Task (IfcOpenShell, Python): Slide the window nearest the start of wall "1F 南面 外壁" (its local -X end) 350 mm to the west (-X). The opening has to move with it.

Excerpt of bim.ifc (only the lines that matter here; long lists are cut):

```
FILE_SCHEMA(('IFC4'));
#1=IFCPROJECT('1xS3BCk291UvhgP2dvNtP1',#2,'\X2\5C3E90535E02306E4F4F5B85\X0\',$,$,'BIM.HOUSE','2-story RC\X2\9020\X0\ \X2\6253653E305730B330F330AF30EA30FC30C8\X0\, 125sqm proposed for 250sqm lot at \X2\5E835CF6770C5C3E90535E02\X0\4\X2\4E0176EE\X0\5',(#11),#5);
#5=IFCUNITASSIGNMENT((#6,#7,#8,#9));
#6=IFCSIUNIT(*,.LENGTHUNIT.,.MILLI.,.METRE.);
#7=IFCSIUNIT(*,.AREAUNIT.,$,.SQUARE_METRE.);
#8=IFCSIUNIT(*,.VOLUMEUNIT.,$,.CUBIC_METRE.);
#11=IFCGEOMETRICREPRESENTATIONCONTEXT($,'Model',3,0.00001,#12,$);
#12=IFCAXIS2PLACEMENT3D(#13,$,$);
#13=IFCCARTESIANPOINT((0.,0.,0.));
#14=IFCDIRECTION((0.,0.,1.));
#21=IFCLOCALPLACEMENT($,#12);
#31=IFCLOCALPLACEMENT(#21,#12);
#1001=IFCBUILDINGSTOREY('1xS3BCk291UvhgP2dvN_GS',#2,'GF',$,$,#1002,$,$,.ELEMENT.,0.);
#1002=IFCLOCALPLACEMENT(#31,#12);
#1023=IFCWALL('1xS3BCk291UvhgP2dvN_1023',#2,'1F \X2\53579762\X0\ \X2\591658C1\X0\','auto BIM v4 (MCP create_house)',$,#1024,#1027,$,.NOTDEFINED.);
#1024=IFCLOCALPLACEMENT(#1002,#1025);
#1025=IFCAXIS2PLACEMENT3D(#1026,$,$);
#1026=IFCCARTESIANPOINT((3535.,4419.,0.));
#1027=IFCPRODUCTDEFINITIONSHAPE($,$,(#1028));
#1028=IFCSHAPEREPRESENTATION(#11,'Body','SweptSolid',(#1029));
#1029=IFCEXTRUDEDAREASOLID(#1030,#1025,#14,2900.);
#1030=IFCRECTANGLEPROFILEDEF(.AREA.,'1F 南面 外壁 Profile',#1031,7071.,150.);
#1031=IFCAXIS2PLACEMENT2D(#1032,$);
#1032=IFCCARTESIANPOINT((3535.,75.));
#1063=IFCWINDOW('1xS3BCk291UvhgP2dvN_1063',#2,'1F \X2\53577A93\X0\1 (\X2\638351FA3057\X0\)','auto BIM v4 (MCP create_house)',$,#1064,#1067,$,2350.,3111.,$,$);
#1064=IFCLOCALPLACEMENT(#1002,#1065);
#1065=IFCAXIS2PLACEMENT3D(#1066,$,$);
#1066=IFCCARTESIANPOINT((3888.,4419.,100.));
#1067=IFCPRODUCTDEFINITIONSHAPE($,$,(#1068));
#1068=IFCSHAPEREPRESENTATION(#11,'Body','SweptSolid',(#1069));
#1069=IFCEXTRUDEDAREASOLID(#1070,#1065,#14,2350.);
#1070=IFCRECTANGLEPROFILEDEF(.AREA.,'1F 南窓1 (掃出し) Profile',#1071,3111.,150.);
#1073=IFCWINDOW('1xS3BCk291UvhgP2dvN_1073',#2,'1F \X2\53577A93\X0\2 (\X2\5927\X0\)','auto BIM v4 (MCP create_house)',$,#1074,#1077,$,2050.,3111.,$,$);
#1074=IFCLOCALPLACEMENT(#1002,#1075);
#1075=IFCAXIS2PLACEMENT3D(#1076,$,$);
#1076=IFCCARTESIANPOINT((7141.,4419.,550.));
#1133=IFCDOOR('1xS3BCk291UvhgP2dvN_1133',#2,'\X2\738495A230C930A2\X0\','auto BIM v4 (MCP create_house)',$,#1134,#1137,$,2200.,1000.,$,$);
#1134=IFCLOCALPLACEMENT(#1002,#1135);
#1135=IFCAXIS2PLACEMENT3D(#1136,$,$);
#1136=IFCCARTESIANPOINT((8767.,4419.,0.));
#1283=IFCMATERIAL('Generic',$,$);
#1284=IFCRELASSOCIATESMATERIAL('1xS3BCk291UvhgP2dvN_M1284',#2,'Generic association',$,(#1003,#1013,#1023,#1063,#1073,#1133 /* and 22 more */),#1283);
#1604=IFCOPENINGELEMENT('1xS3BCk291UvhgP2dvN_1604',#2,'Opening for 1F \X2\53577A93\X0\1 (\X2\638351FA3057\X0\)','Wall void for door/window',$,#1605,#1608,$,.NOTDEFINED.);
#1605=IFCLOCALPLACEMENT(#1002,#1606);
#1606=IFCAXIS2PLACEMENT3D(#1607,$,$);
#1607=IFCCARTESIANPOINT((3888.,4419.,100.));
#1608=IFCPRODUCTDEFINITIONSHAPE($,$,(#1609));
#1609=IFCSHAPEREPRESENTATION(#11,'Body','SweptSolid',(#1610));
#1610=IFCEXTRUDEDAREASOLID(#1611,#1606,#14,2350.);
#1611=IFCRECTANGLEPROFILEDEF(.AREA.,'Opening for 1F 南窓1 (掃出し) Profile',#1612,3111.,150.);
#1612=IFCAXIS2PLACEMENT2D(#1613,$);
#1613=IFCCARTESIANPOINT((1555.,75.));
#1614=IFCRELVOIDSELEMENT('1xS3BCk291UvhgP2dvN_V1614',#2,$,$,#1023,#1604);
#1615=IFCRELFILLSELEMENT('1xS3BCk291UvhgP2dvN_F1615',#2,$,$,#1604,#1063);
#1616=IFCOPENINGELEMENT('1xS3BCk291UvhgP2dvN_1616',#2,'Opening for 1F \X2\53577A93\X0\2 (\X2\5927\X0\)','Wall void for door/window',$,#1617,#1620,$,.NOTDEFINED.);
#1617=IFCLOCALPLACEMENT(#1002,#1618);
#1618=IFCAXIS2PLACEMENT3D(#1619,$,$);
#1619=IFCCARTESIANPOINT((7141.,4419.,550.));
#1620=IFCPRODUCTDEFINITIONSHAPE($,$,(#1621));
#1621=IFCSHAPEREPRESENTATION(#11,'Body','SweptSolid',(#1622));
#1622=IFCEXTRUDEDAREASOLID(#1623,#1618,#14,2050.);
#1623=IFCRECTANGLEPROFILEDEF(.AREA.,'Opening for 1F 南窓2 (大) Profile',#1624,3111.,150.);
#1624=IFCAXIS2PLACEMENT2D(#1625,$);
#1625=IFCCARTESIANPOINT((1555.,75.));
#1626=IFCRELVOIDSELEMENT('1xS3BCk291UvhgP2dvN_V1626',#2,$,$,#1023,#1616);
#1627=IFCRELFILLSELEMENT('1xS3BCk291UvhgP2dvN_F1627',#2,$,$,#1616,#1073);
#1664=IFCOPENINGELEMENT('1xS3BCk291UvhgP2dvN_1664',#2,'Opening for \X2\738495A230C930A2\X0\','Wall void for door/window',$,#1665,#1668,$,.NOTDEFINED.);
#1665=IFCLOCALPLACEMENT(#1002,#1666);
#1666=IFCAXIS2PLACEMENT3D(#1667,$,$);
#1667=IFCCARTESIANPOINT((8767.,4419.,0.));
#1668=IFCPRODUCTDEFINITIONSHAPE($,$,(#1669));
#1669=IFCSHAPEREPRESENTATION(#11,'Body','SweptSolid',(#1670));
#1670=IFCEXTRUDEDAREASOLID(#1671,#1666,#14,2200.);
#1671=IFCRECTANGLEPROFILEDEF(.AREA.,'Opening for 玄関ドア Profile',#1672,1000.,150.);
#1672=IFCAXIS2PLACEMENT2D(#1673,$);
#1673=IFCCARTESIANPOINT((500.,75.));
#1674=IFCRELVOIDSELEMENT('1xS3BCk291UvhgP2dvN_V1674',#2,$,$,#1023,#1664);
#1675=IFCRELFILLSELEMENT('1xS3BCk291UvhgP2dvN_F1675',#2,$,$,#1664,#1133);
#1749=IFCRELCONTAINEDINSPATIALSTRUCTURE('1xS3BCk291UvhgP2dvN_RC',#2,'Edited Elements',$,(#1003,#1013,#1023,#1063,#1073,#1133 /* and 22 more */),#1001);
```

```python
import ifcopenshell
import ifcopenshell.api.geometry
import ifcopenshell.util.placement
import ifcopenshell.util.unit

model = ifcopenshell.open("bim.ifc")
unit_scale = ifcopenshell.util.unit.calculate_unit_scale(model)

window = model.by_guid("1xS3BCk291UvhgP2dvN_1063")
opening = window.FillsVoids[0].RelatingOpeningElement
wall = opening.VoidsElements[0].RelatingBuildingElement

wall_matrix = ifcopenshell.util.placement.get_local_placement(wall.ObjectPlacement)
shift = wall_matrix[:3, 0] * -0.35 / unit_scale
before = ifcopenshell.util.placement.get_local_placement(window.ObjectPlacement)[:3, 3].copy()

# The window is not placed relative to its opening, so move both.
for product in (opening, window):
    matrix = ifcopenshell.util.placement.get_local_placement(product.ObjectPlacement)
    matrix[:3, 3] += shift
    ifcopenshell.api.geometry.edit_object_placement(model, product=product, matrix=matrix, is_si=False)

after = ifcopenshell.util.placement.get_local_placement(window.ObjectPlacement)[:3, 3]
print("window moved by", (after - before).round(3) + 0.0)

model.write("bim-out.ifc")
```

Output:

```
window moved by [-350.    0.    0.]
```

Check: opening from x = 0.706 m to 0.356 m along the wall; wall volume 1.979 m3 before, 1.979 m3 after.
